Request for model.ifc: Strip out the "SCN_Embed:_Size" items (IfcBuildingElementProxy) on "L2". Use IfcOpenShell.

First a look at what the model holds.

```python
import ifcopenshell
import ifcopenshell.util.element

model = ifcopenshell.open("model.ifc")
print(model.schema)
storey = next(s for s in model.by_type("IfcBuildingStorey") if s.Name == "L2")
proxies = [e for e in ifcopenshell.util.element.get_decomposition(storey) if e.is_a("IfcBuildingElementProxy")]
seen = {}
for e in proxies:
    element_type = ifcopenshell.util.element.get_type(e)
    name = element_type.Name if element_type not in (None, e) else None
    seen[name] = seen.get(name, 0) + 1
for name, count in sorted(seen.items(), key=str):
    print(count, "x", name)
```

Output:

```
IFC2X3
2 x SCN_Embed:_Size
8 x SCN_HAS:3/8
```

```python
import ifcopenshell
import ifcopenshell.api.root
import ifcopenshell.util.element

model = ifcopenshell.open("model.ifc")

storey = next(s for s in model.by_type("IfcBuildingStorey") if s.Name == "L2")
proxies = [e for e in ifcopenshell.util.element.get_decomposition(storey) if e.is_a("IfcBuildingElementProxy")]
targets = [e for e in proxies if (t := ifcopenshell.util.element.get_type(e)) not in (None, e) and t.Name == "SCN_Embed:_Size"]

for e in targets:
    ifcopenshell.api.root.remove_product(model, product=e)
print(len(targets), "removed")

model.write("model_rev.ifc")
```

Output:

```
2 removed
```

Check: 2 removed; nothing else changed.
